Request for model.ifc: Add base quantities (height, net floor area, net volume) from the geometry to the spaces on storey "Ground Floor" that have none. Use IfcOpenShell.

First a look at what the model holds.

```python
import ifcopenshell
import ifcopenshell.util.element
import ifcopenshell.util.unit

model = ifcopenshell.open("model.ifc")
print(model.schema)
for unit_type in ("LENGTHUNIT", "AREAUNIT", "VOLUMEUNIT"):
    print(unit_type, ifcopenshell.util.unit.calculate_unit_scale(model, unit_type))
storey = next(s for s in model.by_type("IfcBuildingStorey") if s.Name == "Ground Floor")
spaces = [e for e in ifcopenshell.util.element.get_decomposition(storey) if e.is_a("IfcSpace")]
for e in sorted(spaces, key=lambda e: e.id()):
    print(e.id(), e.is_a(), e.Name, list(ifcopenshell.util.element.get_psets(e, qtos_only=True)), sep=" | ")
```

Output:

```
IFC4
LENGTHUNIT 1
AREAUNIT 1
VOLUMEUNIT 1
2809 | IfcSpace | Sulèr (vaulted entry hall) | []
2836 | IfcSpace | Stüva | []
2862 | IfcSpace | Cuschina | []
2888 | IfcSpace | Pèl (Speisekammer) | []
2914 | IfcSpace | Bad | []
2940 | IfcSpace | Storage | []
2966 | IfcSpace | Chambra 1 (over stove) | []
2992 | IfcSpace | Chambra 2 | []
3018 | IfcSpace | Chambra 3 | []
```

```python
import ifcopenshell
import ifcopenshell.api.pset
import ifcopenshell.geom
import ifcopenshell.util.element
import ifcopenshell.util.shape
import ifcopenshell.util.unit

model = ifcopenshell.open("model.ifc")
unit_scale = ifcopenshell.util.unit.calculate_unit_scale(model)
area_scale = ifcopenshell.util.unit.calculate_unit_scale(model, "AREAUNIT")
volume_scale = ifcopenshell.util.unit.calculate_unit_scale(model, "VOLUMEUNIT")
settings = ifcopenshell.geom.settings()

storey = next(s for s in model.by_type("IfcBuildingStorey") if s.Name == "Ground Floor")
spaces = [e for e in ifcopenshell.util.element.get_decomposition(storey) if e.is_a("IfcSpace")]

for e in sorted(spaces, key=lambda e: e.id()):
    if ifcopenshell.util.element.get_psets(e, qtos_only=True, should_inherit=False):
        continue
    # Geometry comes back in metres, in the element's own axes.
    shape = ifcopenshell.geom.create_shape(settings, e)
    values = {
        "Height": ifcopenshell.util.shape.get_z(shape.geometry) / unit_scale,
        "NetFloorArea": ifcopenshell.util.shape.get_footprint_area(shape.geometry) / area_scale,
        "NetVolume": ifcopenshell.util.shape.get_volume(shape.geometry) / volume_scale,
    }
    qto = ifcopenshell.api.pset.add_qto(model, product=e, name="Qto_SpaceBaseQuantities")
    ifcopenshell.api.pset.edit_qto(model, qto=qto, properties=values)
    print(e.id(), {k: round(v, 3) for k, v in values.items()})

model.write("model_updated.ifc")
```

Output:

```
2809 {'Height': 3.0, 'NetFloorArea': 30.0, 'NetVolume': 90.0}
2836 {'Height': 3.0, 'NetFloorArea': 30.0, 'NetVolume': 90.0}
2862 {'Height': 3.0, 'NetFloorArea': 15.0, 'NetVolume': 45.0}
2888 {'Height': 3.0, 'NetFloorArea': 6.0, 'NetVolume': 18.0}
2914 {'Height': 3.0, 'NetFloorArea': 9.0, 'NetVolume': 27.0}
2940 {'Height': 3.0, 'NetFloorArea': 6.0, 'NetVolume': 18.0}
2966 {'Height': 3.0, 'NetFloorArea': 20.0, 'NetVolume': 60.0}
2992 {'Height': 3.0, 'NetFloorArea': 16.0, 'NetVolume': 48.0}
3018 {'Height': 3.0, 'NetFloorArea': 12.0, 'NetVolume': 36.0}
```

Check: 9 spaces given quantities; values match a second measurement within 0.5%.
